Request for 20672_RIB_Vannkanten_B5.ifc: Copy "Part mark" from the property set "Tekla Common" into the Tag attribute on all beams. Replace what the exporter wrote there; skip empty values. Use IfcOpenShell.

First a look at what the model holds.

```python
import ifcopenshell
import ifcopenshell.util.element

model = ifcopenshell.open("20672_RIB_Vannkanten_B5.ifc")
print(model.schema)
beams = model.by_type("IfcBeam")
print(len(beams), "beams")
for e in beams[:8]:
    source = ifcopenshell.util.element.get_pset(e, "Tekla Common", "Part mark")
    target = e.Tag
    print(e.id(), repr(source), repr(target), sep=" | ")
```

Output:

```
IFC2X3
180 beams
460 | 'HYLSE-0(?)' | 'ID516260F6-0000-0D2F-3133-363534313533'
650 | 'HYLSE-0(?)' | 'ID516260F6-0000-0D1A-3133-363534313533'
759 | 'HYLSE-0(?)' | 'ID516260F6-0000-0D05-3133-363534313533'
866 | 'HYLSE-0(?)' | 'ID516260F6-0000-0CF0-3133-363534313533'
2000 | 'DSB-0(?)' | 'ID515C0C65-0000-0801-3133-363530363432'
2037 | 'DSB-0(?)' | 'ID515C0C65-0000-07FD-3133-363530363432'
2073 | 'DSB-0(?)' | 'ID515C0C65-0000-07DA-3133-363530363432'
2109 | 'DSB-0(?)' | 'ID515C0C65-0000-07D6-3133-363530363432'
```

```python
import ifcopenshell
import ifcopenshell.util.element

model = ifcopenshell.open("20672_RIB_Vannkanten_B5.ifc")

count = 0
for e in model.by_type("IfcBeam"):
    value = ifcopenshell.util.element.get_pset(e, "Tekla Common", "Part mark")
    current = e.Tag
    if not value or not value.strip() or current == value:
        continue
    e.Tag = value
    count += 1

print(count, "beams updated")

model.write("20672_RIB_Vannkanten_B5-out.ifc")
```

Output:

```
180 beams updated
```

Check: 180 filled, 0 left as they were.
